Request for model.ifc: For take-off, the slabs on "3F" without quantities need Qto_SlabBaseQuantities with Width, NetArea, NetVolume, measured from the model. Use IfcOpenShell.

First a look at what the model holds.

```python
import ifcopenshell
import ifcopenshell.util.element
import ifcopenshell.util.unit

model = ifcopenshell.open("model.ifc")
print(model.schema)
for unit_type in ("LENGTHUNIT", "AREAUNIT", "VOLUMEUNIT"):
    print(unit_type, ifcopenshell.util.unit.calculate_unit_scale(model, unit_type))
storey = next(s for s in model.by_type("IfcBuildingStorey") if s.Name == "3F")
slabs = [e for e in ifcopenshell.util.element.get_decomposition(storey) if e.is_a("IfcSlab")]
for e in sorted(slabs, key=lambda e: e.id()):
    print(e.id(), e.is_a(), e.Name, list(ifcopenshell.util.element.get_psets(e, qtos_only=True)), sep=" | ")
```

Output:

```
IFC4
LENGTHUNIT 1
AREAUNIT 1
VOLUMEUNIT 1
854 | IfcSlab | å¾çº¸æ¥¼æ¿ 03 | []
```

```python
import ifcopenshell
import ifcopenshell.api.pset
import ifcopenshell.geom
import ifcopenshell.util.element
import ifcopenshell.util.shape
import ifcopenshell.util.unit

model = ifcopenshell.open("model.ifc")
unit_scale = ifcopenshell.util.unit.calculate_unit_scale(model)
area_scale = ifcopenshell.util.unit.calculate_unit_scale(model, "AREAUNIT")
volume_scale = ifcopenshell.util.unit.calculate_unit_scale(model, "VOLUMEUNIT")
settings = ifcopenshell.geom.settings()

storey = next(s for s in model.by_type("IfcBuildingStorey") if s.Name == "3F")
slabs = [e for e in ifcopenshell.util.element.get_decomposition(storey) if e.is_a("IfcSlab")]

for e in sorted(slabs, key=lambda e: e.id()):
    if ifcopenshell.util.element.get_psets(e, qtos_only=True, should_inherit=False):
        continue
    # Geometry comes back in metres, in the element's own axes.
    shape = ifcopenshell.geom.create_shape(settings, e)
    values = {
        "Width": ifcopenshell.util.shape.get_z(shape.geometry) / unit_scale,
        "NetArea": ifcopenshell.util.shape.get_footprint_area(shape.geometry) / area_scale,
        "NetVolume": ifcopenshell.util.shape.get_volume(shape.geometry) / volume_scale,
    }
    qto = ifcopenshell.api.pset.add_qto(model, product=e, name="Qto_SlabBaseQuantities")
    ifcopenshell.api.pset.edit_qto(model, qto=qto, properties=values)
    print(e.id(), {k: round(v, 3) for k, v in values.items()})

model.write("model_v2.ifc")
```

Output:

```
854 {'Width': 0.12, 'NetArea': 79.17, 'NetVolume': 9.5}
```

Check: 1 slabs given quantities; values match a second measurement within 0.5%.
